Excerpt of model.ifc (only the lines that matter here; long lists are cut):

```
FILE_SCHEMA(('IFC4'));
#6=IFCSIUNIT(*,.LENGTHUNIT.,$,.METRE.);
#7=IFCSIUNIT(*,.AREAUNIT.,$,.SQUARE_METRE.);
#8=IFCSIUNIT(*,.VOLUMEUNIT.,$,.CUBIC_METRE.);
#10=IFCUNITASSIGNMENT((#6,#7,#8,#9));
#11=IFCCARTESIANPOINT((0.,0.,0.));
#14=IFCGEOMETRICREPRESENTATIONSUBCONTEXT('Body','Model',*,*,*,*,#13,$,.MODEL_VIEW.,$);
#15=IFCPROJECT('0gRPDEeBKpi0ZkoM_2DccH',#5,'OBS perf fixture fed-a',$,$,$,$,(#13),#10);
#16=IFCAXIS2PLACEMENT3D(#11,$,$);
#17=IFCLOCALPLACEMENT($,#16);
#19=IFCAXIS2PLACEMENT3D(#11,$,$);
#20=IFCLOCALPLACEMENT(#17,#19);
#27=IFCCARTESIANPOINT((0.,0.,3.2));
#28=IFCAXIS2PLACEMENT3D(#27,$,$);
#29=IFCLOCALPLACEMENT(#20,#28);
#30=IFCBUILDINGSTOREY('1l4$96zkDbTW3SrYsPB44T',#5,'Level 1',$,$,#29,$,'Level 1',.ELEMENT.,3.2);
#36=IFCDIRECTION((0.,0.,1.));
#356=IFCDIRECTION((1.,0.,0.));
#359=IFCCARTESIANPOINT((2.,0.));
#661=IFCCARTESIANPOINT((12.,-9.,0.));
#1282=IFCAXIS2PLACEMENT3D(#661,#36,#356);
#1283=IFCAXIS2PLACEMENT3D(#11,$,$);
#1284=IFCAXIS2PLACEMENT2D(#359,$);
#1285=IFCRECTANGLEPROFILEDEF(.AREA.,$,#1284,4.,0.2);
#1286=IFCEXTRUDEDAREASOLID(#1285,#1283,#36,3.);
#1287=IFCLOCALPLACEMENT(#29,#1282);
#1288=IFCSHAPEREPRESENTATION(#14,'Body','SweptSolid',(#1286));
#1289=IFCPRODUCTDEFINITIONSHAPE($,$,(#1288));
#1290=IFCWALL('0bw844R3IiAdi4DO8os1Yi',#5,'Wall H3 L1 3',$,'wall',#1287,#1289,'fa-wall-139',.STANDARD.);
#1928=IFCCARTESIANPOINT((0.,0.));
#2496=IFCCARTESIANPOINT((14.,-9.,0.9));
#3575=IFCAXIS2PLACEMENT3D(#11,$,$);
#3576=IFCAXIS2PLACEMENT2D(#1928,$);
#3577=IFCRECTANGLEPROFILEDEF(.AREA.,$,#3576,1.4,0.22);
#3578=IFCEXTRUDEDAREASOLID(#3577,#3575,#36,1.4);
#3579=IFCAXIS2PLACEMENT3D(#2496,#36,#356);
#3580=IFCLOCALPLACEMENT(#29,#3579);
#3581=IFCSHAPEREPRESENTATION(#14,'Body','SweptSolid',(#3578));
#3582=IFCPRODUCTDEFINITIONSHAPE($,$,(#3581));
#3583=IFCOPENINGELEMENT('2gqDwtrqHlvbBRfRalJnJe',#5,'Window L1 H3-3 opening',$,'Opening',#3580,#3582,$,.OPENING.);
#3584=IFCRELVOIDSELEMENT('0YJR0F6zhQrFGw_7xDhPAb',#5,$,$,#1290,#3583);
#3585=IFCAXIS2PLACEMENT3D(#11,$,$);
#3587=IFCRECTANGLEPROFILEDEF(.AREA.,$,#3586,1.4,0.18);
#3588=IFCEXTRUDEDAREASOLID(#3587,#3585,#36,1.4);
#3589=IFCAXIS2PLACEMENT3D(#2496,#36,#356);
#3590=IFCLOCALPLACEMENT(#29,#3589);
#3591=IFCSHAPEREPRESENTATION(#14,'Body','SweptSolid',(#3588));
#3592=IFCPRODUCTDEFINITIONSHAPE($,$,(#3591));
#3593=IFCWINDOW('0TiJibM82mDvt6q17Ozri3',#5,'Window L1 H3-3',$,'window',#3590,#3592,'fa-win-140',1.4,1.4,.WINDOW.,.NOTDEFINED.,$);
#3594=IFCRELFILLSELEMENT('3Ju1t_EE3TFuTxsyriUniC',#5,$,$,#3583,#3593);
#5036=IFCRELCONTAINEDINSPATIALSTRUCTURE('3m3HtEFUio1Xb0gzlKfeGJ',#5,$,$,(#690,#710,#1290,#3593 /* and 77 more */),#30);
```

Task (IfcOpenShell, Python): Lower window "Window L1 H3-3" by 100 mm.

```python
import numpy as np
import ifcopenshell
import ifcopenshell.api.geometry
import ifcopenshell.util.placement
import ifcopenshell.util.unit

model = ifcopenshell.open("model.ifc")
unit_scale = ifcopenshell.util.unit.calculate_unit_scale(model)

window = model.by_guid("0TiJibM82mDvt6q17Ozri3")
opening = window.FillsVoids[0].RelatingOpeningElement
dz = -0.1 / unit_scale

shift = np.array([0.0, 0.0, dz])
# The window is not placed relative to its opening, so move both.
for product in (opening, window):
    matrix = ifcopenshell.util.placement.get_local_placement(product.ObjectPlacement)
    matrix[:3, 3] += shift
    ifcopenshell.api.geometry.edit_object_placement(model, product=product, matrix=matrix, is_si=False)

print(f"moved by {dz * unit_scale:+.3f} m")

model.write("model_rev.ifc")
```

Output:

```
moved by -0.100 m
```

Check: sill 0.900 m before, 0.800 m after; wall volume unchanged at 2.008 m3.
